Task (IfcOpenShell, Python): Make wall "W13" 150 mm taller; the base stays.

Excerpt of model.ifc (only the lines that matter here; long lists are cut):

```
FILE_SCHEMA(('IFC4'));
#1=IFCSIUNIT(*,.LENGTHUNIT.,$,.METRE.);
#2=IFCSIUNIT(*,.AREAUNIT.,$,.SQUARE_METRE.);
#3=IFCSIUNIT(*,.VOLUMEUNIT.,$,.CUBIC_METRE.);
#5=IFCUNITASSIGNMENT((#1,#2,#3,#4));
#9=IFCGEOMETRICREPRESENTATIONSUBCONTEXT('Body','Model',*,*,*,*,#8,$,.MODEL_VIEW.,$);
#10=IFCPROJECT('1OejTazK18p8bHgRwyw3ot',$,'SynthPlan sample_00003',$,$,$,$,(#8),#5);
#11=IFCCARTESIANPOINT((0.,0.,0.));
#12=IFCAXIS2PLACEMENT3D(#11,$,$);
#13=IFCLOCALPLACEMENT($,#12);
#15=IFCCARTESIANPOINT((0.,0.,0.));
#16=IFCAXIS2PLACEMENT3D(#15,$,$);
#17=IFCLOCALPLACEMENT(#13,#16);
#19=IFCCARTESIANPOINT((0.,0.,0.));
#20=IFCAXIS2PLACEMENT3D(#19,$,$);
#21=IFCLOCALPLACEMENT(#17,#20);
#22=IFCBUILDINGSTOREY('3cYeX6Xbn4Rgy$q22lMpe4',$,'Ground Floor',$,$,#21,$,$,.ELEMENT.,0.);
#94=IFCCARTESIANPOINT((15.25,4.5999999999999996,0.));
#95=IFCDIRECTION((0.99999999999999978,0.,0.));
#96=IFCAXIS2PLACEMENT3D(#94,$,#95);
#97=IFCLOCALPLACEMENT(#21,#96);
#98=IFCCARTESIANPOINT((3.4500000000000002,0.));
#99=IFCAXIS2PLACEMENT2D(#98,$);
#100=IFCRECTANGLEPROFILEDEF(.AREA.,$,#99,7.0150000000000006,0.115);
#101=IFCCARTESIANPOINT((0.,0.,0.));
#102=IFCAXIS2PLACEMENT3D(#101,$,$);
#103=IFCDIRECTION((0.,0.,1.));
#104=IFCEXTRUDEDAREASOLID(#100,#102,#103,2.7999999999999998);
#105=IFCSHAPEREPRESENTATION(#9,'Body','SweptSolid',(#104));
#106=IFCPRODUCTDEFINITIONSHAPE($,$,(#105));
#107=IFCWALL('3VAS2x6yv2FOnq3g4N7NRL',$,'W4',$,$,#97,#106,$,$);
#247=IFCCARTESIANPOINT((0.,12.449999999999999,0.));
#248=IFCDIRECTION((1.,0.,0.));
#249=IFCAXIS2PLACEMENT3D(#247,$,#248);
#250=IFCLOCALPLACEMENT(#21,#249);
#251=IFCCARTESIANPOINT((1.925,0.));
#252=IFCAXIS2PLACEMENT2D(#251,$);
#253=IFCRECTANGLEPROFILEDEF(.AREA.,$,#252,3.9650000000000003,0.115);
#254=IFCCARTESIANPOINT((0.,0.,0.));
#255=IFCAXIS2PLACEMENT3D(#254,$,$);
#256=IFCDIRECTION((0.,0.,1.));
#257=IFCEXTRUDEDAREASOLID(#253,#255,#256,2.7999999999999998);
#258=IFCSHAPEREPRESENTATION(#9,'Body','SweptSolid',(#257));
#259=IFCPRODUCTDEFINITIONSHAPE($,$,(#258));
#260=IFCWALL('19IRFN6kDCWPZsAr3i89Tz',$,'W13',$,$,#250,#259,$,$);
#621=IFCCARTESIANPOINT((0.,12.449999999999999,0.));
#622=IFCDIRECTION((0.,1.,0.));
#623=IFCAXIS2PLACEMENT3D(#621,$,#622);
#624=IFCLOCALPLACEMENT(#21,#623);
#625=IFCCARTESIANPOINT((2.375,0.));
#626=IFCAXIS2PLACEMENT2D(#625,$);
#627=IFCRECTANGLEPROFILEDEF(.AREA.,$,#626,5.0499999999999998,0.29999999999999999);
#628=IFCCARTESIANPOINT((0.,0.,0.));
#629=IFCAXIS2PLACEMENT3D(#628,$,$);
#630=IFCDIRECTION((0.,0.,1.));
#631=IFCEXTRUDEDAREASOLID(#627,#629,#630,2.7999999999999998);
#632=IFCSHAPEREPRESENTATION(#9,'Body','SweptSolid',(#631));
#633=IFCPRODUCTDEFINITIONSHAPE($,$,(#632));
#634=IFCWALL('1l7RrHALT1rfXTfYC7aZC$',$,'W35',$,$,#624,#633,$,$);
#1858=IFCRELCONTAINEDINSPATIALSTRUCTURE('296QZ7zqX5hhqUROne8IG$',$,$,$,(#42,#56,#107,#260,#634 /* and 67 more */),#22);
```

```python
import ifcopenshell
import ifcopenshell.geom
import ifcopenshell.util.representation
import ifcopenshell.util.shape
import ifcopenshell.util.unit

model = ifcopenshell.open("model.ifc")
unit_scale = ifcopenshell.util.unit.calculate_unit_scale(model)
settings = ifcopenshell.geom.settings()


def volume(element):
    """Net volume in cubic metres, openings subtracted."""
    shape = ifcopenshell.geom.create_shape(settings, element)
    return ifcopenshell.util.shape.get_volume(shape.geometry)


wall = model.by_guid("19IRFN6kDCWPZsAr3i89Tz")
before = volume(wall)

body = ifcopenshell.util.representation.get_representation(wall, "Model", "Body")
solid = body.Items[0]
old_height = solid.Depth
solid.Depth += 0.15 / unit_scale
after = volume(wall)

print(f"height {old_height:g} -> {solid.Depth:g}, volume {before:.3f} -> {after:.3f} m3")

model.write("model_updated.ifc")
```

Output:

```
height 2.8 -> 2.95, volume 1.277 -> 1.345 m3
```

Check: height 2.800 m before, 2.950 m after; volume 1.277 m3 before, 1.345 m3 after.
